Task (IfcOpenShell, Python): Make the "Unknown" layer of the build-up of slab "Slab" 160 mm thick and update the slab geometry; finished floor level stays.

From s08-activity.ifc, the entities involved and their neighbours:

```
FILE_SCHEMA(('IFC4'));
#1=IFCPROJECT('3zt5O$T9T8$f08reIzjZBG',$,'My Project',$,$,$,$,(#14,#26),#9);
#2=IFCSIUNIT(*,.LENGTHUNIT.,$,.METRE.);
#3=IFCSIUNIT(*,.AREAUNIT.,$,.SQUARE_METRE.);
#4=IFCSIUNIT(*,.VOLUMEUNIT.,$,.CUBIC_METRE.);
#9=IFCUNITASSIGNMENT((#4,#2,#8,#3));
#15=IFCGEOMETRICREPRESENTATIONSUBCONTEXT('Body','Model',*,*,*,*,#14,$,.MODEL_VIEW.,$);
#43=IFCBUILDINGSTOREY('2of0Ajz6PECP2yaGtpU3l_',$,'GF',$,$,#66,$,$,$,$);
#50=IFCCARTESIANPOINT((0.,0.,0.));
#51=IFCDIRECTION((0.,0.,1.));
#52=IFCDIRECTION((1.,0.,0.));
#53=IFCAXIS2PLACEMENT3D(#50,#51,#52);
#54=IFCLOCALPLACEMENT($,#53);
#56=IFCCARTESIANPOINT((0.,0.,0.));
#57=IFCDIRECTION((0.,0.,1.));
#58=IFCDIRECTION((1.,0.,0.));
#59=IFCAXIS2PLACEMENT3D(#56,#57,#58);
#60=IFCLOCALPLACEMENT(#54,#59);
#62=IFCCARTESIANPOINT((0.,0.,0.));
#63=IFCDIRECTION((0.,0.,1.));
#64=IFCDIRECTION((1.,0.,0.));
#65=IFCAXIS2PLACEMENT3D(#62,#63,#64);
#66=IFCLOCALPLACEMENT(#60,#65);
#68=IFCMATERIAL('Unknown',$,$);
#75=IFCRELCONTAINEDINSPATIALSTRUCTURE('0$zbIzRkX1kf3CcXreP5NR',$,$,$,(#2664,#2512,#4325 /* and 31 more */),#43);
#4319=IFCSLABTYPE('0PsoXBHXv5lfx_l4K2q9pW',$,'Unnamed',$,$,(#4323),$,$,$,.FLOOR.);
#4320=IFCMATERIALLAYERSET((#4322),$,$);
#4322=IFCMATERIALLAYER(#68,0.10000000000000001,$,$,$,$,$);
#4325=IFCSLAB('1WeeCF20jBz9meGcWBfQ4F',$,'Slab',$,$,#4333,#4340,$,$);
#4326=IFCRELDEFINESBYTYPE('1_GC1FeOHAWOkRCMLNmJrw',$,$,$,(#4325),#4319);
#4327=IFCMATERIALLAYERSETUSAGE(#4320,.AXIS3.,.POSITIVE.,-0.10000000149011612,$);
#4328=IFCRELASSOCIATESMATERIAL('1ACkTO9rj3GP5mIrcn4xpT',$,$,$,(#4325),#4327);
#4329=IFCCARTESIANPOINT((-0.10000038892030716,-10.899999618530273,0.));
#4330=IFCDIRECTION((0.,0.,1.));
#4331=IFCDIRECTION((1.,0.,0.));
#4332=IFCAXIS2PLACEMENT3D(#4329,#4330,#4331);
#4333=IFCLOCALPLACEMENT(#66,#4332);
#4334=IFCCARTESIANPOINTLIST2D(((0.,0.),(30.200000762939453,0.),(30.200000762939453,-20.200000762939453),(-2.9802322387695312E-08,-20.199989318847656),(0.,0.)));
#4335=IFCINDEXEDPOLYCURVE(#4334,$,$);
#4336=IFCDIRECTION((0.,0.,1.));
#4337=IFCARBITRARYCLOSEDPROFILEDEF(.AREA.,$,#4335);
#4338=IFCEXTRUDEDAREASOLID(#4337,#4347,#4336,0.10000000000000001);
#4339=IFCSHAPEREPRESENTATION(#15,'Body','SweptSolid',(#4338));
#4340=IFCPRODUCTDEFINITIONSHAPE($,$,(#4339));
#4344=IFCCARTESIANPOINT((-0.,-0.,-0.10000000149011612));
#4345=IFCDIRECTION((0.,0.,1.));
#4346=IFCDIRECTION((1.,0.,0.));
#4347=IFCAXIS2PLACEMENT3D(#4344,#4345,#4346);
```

```python
import ifcopenshell
import ifcopenshell.util.element
import ifcopenshell.util.representation
import ifcopenshell.util.unit

model = ifcopenshell.open("s08-activity.ifc")
unit_scale = ifcopenshell.util.unit.calculate_unit_scale(model)

layer_set = model.by_id(4320)
layer = next(l for l in layer_set.MaterialLayers if l.Material and l.Material.Name == "Unknown")
change = 0.16 / unit_scale - layer.LayerThickness
layer.LayerThickness += change

# Geometry does not follow the layer set by itself.
slabs = [e for e in ifcopenshell.util.element.get_elements_by_material(model, layer_set) if e.is_a("IfcSlab")]
for slab in sorted(slabs, key=lambda e: e.id()):
    body = ifcopenshell.util.representation.get_representation(slab, "Model", "Body")
    solid = body.Items[0]
    old_depth = solid.Depth
    solid.Depth += change
    # Extruded upwards: lower the start of the extrusion so the top stays.
    x, y, z = solid.Position.Location.Coordinates
    solid.Position.Location = model.createIfcCartesianPoint((x, y, z - change))
    print(slab.id(), f"{old_depth:g} -> {solid.Depth:g}")

# The layers are counted up from the underside, which has moved.
for usage in {ifcopenshell.util.element.get_material(slab) for slab in slabs}:
    usage.OffsetFromReferenceLine -= change

model.write("s08-activity-out.ifc")
```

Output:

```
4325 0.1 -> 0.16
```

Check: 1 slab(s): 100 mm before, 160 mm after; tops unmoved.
